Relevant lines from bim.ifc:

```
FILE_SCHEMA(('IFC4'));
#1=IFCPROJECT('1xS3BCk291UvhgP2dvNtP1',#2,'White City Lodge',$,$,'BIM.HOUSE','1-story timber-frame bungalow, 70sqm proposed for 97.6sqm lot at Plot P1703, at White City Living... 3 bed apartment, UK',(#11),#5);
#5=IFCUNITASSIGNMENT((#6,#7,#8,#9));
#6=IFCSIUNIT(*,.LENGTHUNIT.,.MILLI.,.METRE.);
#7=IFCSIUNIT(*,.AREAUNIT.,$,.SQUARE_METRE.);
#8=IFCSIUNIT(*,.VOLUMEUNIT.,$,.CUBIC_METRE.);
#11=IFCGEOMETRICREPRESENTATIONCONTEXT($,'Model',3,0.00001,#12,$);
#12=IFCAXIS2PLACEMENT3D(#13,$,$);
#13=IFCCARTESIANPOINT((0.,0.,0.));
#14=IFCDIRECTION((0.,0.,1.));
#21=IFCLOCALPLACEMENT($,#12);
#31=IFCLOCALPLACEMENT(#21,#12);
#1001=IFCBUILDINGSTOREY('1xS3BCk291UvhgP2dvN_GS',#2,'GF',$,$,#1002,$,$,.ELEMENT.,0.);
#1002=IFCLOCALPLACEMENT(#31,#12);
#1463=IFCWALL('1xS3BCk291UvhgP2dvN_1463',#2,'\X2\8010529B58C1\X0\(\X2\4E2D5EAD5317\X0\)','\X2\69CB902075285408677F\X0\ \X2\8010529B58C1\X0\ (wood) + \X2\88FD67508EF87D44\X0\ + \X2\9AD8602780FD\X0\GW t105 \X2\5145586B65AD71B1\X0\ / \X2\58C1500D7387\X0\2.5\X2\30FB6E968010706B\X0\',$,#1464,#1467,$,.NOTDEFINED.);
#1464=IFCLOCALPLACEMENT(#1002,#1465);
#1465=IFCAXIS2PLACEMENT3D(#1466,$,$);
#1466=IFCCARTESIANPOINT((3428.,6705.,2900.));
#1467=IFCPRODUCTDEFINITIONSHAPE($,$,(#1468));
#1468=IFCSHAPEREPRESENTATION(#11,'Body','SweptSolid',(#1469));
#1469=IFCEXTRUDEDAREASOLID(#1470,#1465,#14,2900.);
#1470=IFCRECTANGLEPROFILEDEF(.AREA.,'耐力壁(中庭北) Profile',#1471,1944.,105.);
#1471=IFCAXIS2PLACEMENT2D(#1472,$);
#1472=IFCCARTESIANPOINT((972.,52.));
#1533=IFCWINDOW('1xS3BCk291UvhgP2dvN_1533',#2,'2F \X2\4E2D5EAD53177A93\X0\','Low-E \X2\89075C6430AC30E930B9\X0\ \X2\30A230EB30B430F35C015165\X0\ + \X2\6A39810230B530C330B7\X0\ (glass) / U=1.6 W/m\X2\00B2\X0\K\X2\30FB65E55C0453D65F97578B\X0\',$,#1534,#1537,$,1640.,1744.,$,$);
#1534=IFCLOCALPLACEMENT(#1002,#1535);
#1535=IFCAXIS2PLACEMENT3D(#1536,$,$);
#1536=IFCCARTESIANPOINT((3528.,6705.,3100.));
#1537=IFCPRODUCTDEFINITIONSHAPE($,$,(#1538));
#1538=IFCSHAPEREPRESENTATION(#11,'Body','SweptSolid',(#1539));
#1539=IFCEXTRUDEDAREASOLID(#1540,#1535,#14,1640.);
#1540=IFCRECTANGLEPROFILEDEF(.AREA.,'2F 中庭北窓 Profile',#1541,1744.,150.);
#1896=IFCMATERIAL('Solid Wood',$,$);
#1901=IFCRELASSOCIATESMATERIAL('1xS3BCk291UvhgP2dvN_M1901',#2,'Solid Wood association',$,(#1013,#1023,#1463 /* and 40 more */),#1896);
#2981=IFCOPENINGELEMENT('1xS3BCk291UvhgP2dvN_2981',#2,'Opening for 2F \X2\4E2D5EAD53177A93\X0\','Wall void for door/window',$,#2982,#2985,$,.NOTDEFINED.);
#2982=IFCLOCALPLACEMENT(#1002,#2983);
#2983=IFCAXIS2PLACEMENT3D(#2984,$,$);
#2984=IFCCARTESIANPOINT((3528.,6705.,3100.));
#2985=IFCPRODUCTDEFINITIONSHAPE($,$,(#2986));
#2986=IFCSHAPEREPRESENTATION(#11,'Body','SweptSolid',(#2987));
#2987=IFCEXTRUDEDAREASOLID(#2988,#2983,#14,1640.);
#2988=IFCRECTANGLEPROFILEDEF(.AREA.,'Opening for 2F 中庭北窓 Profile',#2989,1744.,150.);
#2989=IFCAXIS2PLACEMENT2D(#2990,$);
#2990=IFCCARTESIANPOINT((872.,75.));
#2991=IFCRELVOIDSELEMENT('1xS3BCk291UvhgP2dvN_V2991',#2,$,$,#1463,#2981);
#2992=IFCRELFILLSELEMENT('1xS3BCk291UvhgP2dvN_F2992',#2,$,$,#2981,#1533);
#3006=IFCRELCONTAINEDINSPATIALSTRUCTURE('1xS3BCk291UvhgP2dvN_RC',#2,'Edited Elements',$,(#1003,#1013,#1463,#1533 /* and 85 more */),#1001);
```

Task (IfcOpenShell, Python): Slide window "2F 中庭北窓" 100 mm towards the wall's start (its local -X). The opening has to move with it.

```python
import ifcopenshell
import ifcopenshell.api.geometry
import ifcopenshell.util.placement
import ifcopenshell.util.unit

model = ifcopenshell.open("bim.ifc")
unit_scale = ifcopenshell.util.unit.calculate_unit_scale(model)

window = model.by_id(1533)
opening = window.FillsVoids[0].RelatingOpeningElement
wall = opening.VoidsElements[0].RelatingBuildingElement

wall_matrix = ifcopenshell.util.placement.get_local_placement(wall.ObjectPlacement)
shift = wall_matrix[:3, 0] * -0.1 / unit_scale
before = ifcopenshell.util.placement.get_local_placement(window.ObjectPlacement)[:3, 3].copy()

# The window is not placed relative to its opening, so move both.
for product in (opening, window):
    matrix = ifcopenshell.util.placement.get_local_placement(product.ObjectPlacement)
    matrix[:3, 3] += shift
    ifcopenshell.api.geometry.edit_object_placement(model, product=product, matrix=matrix, is_si=False)

after = ifcopenshell.util.placement.get_local_placement(window.ObjectPlacement)[:3, 3]
print("window moved by", (after - before).round(3) + 0.0)

model.write("bim_rev.ifc")
```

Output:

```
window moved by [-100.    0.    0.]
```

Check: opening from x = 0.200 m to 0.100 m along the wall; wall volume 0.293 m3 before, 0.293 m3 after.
